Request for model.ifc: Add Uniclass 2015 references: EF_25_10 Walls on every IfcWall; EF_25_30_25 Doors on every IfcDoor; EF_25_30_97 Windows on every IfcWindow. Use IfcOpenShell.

First a look at what the model holds.

```python
import ifcopenshell

model = ifcopenshell.open("model.ifc")
print(model.schema)
print("classifications:", [c.Name for c in model.by_type("IfcClassification")])
for ifc_class in ("IfcDoor", "IfcRoof", "IfcStair", "IfcWall", "IfcWindow"):
    print(ifc_class, len(model.by_type(ifc_class)))
```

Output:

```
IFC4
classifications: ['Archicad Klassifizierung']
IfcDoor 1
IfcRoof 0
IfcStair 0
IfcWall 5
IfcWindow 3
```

```python
import ifcopenshell
import ifcopenshell.api.classification

model = ifcopenshell.open("model.ifc")

system = ifcopenshell.api.classification.add_classification(model, classification="Uniclass 2015")

codes = {
    "IfcWall": ("EF_25_10", "Walls"),
    "IfcDoor": ("EF_25_30_25", "Doors"),
    "IfcWindow": ("EF_25_30_97", "Windows"),
}
for ifc_class, (code, name) in codes.items():
    products = model.by_type(ifc_class)
    ifcopenshell.api.classification.add_reference(
        model, products=products, classification=system, identification=code, name=name
    )
    print(code, len(products))

model.write("model_rev.ifc")
```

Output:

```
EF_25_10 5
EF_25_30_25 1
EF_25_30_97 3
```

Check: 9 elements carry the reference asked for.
